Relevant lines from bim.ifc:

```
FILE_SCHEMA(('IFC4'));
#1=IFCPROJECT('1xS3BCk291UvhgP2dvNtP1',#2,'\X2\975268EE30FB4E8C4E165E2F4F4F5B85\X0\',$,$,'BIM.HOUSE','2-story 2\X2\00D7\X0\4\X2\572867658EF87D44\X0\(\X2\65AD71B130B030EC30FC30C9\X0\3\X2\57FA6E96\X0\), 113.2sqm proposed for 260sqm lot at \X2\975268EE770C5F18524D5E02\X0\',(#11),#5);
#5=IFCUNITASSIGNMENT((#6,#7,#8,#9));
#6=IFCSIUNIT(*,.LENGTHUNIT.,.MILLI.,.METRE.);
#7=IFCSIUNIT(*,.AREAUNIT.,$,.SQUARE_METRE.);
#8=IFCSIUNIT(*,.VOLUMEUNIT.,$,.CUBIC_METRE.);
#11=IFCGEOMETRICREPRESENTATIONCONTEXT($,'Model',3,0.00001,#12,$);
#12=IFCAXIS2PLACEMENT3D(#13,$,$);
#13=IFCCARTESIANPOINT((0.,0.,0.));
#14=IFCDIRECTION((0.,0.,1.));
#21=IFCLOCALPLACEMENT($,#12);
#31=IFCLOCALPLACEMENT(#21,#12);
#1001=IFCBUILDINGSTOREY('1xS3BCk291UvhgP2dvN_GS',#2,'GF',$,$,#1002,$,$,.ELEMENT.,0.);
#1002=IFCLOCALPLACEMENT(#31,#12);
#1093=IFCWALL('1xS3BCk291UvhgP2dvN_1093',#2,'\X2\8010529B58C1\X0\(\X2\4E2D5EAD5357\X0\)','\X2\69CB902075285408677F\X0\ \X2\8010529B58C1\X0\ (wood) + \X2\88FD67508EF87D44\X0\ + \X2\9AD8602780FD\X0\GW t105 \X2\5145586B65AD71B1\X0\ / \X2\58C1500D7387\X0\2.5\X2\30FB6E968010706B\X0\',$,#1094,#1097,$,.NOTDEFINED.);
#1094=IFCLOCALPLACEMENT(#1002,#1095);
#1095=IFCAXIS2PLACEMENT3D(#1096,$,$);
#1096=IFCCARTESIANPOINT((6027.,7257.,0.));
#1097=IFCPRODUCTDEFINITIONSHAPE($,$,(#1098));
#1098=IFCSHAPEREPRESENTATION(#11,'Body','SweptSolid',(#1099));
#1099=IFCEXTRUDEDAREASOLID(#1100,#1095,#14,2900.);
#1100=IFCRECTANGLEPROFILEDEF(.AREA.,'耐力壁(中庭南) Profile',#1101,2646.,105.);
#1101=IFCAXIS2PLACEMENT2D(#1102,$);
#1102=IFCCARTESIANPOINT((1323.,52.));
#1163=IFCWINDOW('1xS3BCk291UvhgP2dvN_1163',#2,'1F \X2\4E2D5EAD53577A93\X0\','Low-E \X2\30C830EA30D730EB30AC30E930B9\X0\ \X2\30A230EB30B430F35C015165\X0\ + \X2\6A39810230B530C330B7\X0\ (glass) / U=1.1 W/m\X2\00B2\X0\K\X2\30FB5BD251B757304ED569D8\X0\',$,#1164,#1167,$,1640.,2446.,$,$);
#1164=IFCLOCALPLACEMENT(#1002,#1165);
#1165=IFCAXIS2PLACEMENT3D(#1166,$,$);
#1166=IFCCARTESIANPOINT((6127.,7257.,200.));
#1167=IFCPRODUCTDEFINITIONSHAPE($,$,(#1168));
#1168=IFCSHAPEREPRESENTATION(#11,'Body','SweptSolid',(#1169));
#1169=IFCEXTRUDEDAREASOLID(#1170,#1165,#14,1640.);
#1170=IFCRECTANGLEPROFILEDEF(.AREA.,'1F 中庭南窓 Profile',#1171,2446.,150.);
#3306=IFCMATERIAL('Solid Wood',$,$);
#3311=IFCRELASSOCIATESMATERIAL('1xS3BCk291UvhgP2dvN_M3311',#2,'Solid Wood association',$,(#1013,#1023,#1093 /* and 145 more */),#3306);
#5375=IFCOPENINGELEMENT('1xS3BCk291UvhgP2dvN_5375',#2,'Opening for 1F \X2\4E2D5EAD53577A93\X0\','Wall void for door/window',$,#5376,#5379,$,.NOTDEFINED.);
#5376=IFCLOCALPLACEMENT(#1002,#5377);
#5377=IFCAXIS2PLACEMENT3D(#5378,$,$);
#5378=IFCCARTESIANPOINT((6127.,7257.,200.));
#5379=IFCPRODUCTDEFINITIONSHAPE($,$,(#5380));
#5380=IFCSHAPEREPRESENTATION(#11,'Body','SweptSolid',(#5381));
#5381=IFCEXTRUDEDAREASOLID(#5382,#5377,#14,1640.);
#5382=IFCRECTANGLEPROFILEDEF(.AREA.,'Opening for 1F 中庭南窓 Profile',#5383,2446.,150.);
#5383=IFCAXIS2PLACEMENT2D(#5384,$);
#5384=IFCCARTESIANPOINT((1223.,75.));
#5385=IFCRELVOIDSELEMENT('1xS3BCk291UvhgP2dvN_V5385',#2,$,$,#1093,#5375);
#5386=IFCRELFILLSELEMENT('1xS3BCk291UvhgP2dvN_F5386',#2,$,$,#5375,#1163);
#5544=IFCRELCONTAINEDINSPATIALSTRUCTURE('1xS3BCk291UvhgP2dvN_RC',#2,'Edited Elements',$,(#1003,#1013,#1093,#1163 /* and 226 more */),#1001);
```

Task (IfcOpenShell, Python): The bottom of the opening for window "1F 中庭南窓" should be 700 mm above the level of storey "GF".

```python
import numpy as np
import ifcopenshell
import ifcopenshell.api.geometry
import ifcopenshell.geom
import ifcopenshell.util.element
import ifcopenshell.util.placement
import ifcopenshell.util.shape
import ifcopenshell.util.unit

model = ifcopenshell.open("bim.ifc")
unit_scale = ifcopenshell.util.unit.calculate_unit_scale(model)

window = model.by_guid("1xS3BCk291UvhgP2dvN_1163")
opening = window.FillsVoids[0].RelatingOpeningElement
storey = ifcopenshell.util.element.get_container(window, ifc_class="IfcBuildingStorey")
level = ifcopenshell.util.placement.get_local_placement(storey.ObjectPlacement)[2, 3]

# The opening's origin need not be at the sill, so measure its lowest point.
shape = ifcopenshell.geom.create_shape(ifcopenshell.geom.settings(), opening)
bottom = ifcopenshell.util.shape.get_shape_bottom_elevation(shape, shape.geometry) / unit_scale
dz = level + 0.7 / unit_scale - bottom

shift = np.array([0.0, 0.0, dz])
# The window is not placed relative to its opening, so move both.
for product in (opening, window):
    matrix = ifcopenshell.util.placement.get_local_placement(product.ObjectPlacement)
    matrix[:3, 3] += shift
    ifcopenshell.api.geometry.edit_object_placement(model, product=product, matrix=matrix, is_si=False)

print(f"moved by {dz * unit_scale:+.3f} m")

model.write("bim_edited.ifc")
```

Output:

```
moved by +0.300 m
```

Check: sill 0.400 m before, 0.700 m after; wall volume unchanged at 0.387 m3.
